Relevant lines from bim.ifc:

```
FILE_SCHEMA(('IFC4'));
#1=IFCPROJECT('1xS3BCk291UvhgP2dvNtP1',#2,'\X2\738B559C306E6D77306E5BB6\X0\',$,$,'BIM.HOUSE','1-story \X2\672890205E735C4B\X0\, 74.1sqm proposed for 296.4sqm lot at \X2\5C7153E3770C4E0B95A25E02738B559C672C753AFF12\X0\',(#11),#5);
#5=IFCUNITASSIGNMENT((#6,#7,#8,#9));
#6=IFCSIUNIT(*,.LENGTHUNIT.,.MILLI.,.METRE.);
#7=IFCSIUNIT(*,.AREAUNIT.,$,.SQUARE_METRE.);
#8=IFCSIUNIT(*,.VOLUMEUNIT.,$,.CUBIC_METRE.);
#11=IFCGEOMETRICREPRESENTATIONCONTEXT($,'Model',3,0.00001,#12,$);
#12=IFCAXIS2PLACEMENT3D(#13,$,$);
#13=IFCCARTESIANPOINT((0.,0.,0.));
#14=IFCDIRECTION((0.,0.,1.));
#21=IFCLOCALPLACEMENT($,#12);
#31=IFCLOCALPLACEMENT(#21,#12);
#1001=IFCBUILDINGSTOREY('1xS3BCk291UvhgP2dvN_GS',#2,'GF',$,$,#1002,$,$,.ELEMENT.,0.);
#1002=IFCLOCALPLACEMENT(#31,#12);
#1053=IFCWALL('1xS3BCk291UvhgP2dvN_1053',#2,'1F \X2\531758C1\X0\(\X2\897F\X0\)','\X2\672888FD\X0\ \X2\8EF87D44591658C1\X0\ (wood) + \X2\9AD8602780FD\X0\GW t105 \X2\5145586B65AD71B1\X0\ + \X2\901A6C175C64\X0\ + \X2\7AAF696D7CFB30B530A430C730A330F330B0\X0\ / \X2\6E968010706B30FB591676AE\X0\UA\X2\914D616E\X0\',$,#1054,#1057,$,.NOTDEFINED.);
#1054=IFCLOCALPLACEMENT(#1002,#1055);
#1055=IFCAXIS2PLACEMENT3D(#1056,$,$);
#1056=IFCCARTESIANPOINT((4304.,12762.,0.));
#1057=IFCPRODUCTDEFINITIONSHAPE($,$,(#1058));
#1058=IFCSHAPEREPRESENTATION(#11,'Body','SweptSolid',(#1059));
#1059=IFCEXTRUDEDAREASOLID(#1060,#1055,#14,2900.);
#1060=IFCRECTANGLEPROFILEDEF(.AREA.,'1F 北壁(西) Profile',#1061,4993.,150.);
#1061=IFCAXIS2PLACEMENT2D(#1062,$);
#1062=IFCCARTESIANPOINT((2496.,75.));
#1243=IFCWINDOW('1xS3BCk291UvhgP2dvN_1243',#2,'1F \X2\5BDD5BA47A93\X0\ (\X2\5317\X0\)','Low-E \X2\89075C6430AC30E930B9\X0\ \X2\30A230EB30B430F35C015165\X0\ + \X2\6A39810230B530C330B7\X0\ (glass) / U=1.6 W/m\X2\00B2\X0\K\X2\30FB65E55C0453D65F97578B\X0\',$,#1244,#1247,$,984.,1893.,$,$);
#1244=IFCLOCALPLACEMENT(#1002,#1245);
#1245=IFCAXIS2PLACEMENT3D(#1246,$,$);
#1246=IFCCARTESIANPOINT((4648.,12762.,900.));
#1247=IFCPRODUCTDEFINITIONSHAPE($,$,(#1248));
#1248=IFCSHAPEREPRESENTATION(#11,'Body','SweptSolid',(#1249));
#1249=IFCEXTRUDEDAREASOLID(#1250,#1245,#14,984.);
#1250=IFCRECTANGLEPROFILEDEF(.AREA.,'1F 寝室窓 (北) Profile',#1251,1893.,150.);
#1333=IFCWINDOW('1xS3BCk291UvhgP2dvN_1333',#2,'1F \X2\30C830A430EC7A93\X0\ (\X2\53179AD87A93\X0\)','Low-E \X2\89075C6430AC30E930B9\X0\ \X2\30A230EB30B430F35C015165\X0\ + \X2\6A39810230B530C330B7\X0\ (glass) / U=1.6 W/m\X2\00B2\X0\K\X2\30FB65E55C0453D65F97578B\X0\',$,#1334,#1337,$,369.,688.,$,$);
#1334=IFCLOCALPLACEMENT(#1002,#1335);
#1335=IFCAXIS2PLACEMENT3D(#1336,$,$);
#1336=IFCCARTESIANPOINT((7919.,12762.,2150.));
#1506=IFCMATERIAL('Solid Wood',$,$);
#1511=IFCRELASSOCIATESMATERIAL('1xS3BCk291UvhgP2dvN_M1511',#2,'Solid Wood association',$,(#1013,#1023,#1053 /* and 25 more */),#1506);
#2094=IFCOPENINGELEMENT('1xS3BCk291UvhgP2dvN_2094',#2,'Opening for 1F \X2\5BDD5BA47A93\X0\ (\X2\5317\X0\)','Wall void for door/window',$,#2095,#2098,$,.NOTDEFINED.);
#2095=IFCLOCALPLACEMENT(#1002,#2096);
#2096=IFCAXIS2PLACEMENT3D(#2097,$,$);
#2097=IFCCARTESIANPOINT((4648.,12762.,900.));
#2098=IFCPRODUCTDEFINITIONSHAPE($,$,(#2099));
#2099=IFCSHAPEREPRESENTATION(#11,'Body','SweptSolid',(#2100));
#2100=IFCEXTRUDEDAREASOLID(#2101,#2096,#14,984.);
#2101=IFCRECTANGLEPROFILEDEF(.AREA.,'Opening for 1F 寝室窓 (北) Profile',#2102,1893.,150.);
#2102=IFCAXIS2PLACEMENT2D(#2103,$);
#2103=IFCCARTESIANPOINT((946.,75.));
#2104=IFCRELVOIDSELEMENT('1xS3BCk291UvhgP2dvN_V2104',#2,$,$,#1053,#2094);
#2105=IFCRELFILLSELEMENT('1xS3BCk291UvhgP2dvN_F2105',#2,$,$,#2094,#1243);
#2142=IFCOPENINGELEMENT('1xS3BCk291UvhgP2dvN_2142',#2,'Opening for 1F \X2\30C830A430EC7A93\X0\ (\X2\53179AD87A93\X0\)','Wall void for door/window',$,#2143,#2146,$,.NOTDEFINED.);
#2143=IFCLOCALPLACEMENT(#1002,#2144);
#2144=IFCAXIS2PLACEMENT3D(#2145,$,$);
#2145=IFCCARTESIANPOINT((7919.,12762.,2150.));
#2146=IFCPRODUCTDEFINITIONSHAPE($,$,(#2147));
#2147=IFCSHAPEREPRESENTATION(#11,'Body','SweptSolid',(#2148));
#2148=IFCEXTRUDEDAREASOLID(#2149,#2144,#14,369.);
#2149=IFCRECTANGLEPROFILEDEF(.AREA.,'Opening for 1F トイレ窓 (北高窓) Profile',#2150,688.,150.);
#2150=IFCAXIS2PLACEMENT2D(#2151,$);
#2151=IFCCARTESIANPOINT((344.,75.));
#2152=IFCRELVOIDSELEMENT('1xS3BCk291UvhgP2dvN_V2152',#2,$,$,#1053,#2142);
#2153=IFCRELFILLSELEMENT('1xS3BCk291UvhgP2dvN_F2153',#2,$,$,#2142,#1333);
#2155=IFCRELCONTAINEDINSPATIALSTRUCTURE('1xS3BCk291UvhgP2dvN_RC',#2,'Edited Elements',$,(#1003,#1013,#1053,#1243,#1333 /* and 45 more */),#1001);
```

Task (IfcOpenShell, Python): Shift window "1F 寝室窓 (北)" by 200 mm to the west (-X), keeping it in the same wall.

```python
import ifcopenshell
import ifcopenshell.api.geometry
import ifcopenshell.util.placement
import ifcopenshell.util.unit

model = ifcopenshell.open("bim.ifc")
unit_scale = ifcopenshell.util.unit.calculate_unit_scale(model)

window = model.by_guid("1xS3BCk291UvhgP2dvN_1243")
opening = window.FillsVoids[0].RelatingOpeningElement
wall = opening.VoidsElements[0].RelatingBuildingElement

wall_matrix = ifcopenshell.util.placement.get_local_placement(wall.ObjectPlacement)
shift = wall_matrix[:3, 0] * -0.2 / unit_scale
before = ifcopenshell.util.placement.get_local_placement(window.ObjectPlacement)[:3, 3].copy()

# The window is not placed relative to its opening, so move both.
for product in (opening, window):
    matrix = ifcopenshell.util.placement.get_local_placement(product.ObjectPlacement)
    matrix[:3, 3] += shift
    ifcopenshell.api.geometry.edit_object_placement(model, product=product, matrix=matrix, is_si=False)

after = ifcopenshell.util.placement.get_local_placement(window.ObjectPlacement)[:3, 3]
print("window moved by", (after - before).round(3) + 0.0)

model.write("bim_edited.ifc")
```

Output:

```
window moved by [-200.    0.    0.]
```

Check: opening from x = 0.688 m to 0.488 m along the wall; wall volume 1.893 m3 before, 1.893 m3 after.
